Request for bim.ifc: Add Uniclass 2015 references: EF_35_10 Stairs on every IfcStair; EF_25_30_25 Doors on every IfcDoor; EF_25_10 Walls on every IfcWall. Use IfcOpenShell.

First a look at what the model holds.

```python
import ifcopenshell

model = ifcopenshell.open("bim.ifc")
print(model.schema)
print("classifications:", [c.Name for c in model.by_type("IfcClassification")])
for ifc_class in ("IfcDoor", "IfcRoof", "IfcStair", "IfcWall", "IfcWindow"):
    print(ifc_class, len(model.by_type(ifc_class)))
```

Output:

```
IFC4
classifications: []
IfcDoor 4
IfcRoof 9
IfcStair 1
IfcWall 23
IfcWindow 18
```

```python
import ifcopenshell
import ifcopenshell.api.classification

model = ifcopenshell.open("bim.ifc")

system = ifcopenshell.api.classification.add_classification(model, classification="Uniclass 2015")

codes = {
    "IfcStair": ("EF_35_10", "Stairs"),
    "IfcDoor": ("EF_25_30_25", "Doors"),
    "IfcWall": ("EF_25_10", "Walls"),
}
for ifc_class, (code, name) in codes.items():
    products = model.by_type(ifc_class)
    ifcopenshell.api.classification.add_reference(
        model, products=products, classification=system, identification=code, name=name
    )
    print(code, len(products))

model.write("bim_updated.ifc")
```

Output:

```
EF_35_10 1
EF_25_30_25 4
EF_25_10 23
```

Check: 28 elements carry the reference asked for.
